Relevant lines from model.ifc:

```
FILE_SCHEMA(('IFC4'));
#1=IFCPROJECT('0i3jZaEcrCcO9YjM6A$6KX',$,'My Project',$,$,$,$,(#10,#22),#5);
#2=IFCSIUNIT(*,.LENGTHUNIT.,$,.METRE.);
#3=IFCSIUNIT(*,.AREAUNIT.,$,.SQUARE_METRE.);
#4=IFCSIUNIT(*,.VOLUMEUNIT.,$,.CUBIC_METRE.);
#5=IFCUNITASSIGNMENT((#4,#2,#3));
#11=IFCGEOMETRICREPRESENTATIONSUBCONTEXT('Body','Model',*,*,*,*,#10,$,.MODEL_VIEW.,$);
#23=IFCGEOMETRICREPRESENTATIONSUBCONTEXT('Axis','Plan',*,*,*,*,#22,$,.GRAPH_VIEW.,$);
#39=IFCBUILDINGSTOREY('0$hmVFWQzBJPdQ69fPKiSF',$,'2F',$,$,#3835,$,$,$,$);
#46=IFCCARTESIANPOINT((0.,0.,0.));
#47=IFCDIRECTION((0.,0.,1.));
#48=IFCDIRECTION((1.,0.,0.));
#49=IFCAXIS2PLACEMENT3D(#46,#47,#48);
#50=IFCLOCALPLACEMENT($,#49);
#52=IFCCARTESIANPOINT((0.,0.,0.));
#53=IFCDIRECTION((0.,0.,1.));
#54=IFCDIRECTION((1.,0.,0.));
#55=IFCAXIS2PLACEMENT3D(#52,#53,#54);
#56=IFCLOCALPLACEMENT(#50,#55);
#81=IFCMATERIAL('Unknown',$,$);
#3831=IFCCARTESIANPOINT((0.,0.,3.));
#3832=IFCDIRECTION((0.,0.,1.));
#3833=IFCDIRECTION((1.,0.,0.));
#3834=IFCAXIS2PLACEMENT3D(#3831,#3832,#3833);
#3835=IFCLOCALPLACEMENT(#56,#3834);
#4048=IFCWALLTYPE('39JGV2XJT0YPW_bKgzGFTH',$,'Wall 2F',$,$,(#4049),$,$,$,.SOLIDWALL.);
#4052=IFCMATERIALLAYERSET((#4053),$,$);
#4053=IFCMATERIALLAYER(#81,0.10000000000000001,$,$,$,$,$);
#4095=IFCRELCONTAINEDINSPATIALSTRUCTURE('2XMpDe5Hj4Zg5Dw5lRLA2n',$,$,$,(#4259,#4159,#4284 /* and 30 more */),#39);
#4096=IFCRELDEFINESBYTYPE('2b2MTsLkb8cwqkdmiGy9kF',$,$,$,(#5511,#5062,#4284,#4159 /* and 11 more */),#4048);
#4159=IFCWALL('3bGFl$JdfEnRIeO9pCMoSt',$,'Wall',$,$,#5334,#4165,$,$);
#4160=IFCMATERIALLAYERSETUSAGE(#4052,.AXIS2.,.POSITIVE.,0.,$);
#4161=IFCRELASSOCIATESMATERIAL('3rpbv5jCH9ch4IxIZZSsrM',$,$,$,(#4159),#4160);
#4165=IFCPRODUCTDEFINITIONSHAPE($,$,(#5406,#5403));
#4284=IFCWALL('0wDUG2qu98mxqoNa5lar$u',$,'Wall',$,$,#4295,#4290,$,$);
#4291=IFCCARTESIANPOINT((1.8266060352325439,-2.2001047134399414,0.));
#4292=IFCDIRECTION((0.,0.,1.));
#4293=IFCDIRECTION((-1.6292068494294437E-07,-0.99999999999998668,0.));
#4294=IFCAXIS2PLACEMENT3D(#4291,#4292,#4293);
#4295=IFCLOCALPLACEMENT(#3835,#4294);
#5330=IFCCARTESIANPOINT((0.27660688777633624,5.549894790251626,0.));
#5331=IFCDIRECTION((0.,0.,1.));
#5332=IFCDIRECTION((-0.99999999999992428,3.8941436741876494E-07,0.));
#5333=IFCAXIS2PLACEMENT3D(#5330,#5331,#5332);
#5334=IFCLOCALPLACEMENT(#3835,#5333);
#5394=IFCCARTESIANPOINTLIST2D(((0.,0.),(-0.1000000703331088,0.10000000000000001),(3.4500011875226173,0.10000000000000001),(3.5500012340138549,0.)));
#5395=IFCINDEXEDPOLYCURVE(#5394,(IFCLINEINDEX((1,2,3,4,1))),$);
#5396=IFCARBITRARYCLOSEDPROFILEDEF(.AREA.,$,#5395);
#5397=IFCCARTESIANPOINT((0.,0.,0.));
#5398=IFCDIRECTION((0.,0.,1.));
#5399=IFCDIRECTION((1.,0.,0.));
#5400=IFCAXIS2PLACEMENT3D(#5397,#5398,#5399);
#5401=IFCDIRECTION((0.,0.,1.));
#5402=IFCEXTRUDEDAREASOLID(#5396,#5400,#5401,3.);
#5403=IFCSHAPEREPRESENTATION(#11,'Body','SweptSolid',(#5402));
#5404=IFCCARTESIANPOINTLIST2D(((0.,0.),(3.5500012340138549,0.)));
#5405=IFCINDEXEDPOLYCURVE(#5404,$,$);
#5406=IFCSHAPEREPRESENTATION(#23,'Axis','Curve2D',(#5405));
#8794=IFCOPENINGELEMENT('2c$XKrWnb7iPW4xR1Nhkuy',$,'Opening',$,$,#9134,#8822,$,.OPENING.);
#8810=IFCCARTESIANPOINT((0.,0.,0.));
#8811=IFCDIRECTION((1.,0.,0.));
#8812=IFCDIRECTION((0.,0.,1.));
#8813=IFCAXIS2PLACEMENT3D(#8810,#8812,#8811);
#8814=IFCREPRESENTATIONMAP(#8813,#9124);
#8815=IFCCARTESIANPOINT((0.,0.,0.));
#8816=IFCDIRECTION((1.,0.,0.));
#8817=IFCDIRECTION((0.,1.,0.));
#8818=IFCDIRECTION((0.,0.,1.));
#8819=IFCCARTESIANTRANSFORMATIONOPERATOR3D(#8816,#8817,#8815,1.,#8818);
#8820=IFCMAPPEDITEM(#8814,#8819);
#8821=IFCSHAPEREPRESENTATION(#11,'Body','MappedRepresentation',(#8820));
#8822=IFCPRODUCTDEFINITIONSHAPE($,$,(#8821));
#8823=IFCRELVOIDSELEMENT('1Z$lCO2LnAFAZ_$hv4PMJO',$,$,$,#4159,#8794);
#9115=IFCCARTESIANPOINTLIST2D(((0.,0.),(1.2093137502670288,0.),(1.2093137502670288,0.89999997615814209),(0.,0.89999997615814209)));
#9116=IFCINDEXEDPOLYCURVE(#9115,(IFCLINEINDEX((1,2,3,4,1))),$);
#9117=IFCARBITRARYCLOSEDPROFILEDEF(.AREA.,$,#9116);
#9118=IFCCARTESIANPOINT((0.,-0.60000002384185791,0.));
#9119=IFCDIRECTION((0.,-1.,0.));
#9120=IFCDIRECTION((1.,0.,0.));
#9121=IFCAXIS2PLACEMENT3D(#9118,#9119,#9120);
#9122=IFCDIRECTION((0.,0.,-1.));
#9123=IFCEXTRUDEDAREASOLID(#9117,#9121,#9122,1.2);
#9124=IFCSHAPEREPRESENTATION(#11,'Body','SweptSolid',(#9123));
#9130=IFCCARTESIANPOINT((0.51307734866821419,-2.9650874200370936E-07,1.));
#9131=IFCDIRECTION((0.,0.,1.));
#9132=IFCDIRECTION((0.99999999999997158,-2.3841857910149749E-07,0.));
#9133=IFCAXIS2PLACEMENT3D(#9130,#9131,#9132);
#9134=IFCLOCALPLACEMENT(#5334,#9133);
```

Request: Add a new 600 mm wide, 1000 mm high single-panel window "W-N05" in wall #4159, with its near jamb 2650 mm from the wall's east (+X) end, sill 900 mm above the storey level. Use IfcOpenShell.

```python
import numpy as np
import ifcopenshell
import ifcopenshell.api.feature
import ifcopenshell.api.geometry
import ifcopenshell.api.root
import ifcopenshell.api.spatial
import ifcopenshell.geom
import ifcopenshell.util.element
import ifcopenshell.util.placement
import ifcopenshell.util.representation
import ifcopenshell.util.shape
import ifcopenshell.util.unit

model = ifcopenshell.open("model.ifc")
unit_scale = ifcopenshell.util.unit.calculate_unit_scale(model)
settings = ifcopenshell.geom.settings()


def volume(element):
    """Net volume in cubic metres, openings subtracted."""
    shape = ifcopenshell.geom.create_shape(settings, element)
    return ifcopenshell.util.shape.get_volume(shape.geometry)


wall = model.by_guid("3bGFl$JdfEnRIeO9pCMoSt")
storey = ifcopenshell.util.element.get_container(wall, ifc_class="IfcBuildingStorey")
context = ifcopenshell.util.representation.get_context(model, "Model", "Body", "MODEL_VIEW")
before = volume(wall)

width, height, from_end, sill = 0.6, 1, 2.65, 0.9  # metres

# The wall runs along its own X axis, and the end named is its -X end.
wall_shape = ifcopenshell.geom.create_shape(settings, wall)
x, y, z = ifcopenshell.util.shape.get_vertices(wall_shape.geometry).T
start = x.min() + from_end
face, thickness = float(y.min()), float(y.max() - y.min())
wall_matrix = ifcopenshell.util.placement.get_local_placement(wall.ObjectPlacement)
level = ifcopenshell.util.placement.get_local_placement(storey.ObjectPlacement)[2, 3]


def in_wall(x, y):
    """Placement at x, y metres in the wall's axes, at sill height."""
    matrix = wall_matrix.copy()
    matrix[:, 3] = wall_matrix @ np.array([x / unit_scale, y / unit_scale, 0.0, 1.0])
    matrix[2, 3] = level + sill / unit_scale
    return matrix


# Opening: a box that overshoots both wall faces by 50 mm.
opening = ifcopenshell.api.root.create_entity(model, ifc_class="IfcOpeningElement", predefined_type="OPENING")
box = ifcopenshell.api.geometry.add_wall_representation(
    model, context=context, length=width, height=height, thickness=thickness + 0.1
)
ifcopenshell.api.geometry.assign_representation(model, product=opening, representation=box)
ifcopenshell.api.geometry.edit_object_placement(model, product=opening, matrix=in_wall(start, face - 0.05), is_si=False)
ifcopenshell.api.feature.add_feature(model, feature=opening, element=wall)

window = ifcopenshell.api.root.create_entity(model, ifc_class="IfcWindow", name="W-N05", predefined_type="WINDOW")
window.OverallWidth, window.OverallHeight = width / unit_scale, height / unit_scale
window.PartitioningType = "SINGLE_PANEL"
body = ifcopenshell.api.geometry.add_window_representation(
    model,
    context=context,
    overall_width=window.OverallWidth,
    overall_height=window.OverallHeight,
    partition_type="SINGLE_PANEL",
)
ifcopenshell.api.geometry.assign_representation(model, product=window, representation=body)
ifcopenshell.api.spatial.assign_container(model, products=[window], relating_structure=storey)
ifcopenshell.api.feature.add_filling(model, opening=opening, element=window)

# Centre the window in the wall's thickness.
ifcopenshell.api.geometry.edit_object_placement(model, product=window, matrix=in_wall(start, face), is_si=False)
window_shape = ifcopenshell.geom.create_shape(settings, window)
depth = ifcopenshell.util.shape.get_vertices(window_shape.geometry)[:, 1]
offset = face + thickness / 2 - (depth.min() + depth.max()) / 2
ifcopenshell.api.geometry.edit_object_placement(model, product=window, matrix=in_wall(start, offset), is_si=False)

after = volume(wall)

print(f"wall volume {before:.3f} -> {after:.3f} m3")

model.write("model_updated.ifc")
```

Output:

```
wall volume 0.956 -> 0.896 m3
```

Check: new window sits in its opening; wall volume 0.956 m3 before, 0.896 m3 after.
